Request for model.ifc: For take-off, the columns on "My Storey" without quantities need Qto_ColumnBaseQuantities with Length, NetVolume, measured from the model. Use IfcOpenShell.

First a look at what the model holds.

```python
import ifcopenshell
import ifcopenshell.util.element
import ifcopenshell.util.unit

model = ifcopenshell.open("model.ifc")
print(model.schema)
for unit_type in ("LENGTHUNIT", "AREAUNIT", "VOLUMEUNIT"):
    print(unit_type, ifcopenshell.util.unit.calculate_unit_scale(model, unit_type))
storey = next(s for s in model.by_type("IfcBuildingStorey") if s.Name == "My Storey")
columns = [e for e in ifcopenshell.util.element.get_decomposition(storey) if e.is_a("IfcColumn")]
for e in sorted(columns, key=lambda e: e.id()):
    print(e.id(), e.is_a(), e.Name, list(ifcopenshell.util.element.get_psets(e, qtos_only=True)), sep=" | ")
```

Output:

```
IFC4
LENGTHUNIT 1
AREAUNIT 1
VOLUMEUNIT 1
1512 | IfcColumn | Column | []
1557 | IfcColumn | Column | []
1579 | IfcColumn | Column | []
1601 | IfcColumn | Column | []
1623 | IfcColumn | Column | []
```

```python
import ifcopenshell
import ifcopenshell.api.pset
import ifcopenshell.geom
import ifcopenshell.util.element
import ifcopenshell.util.shape
import ifcopenshell.util.unit

model = ifcopenshell.open("model.ifc")
unit_scale = ifcopenshell.util.unit.calculate_unit_scale(model)
volume_scale = ifcopenshell.util.unit.calculate_unit_scale(model, "VOLUMEUNIT")
settings = ifcopenshell.geom.settings()

storey = next(s for s in model.by_type("IfcBuildingStorey") if s.Name == "My Storey")
columns = [e for e in ifcopenshell.util.element.get_decomposition(storey) if e.is_a("IfcColumn")]

for e in sorted(columns, key=lambda e: e.id()):
    if ifcopenshell.util.element.get_psets(e, qtos_only=True, should_inherit=False):
        continue
    # Geometry comes back in metres, in the element's own axes.
    shape = ifcopenshell.geom.create_shape(settings, e)
    values = {
        "Length": ifcopenshell.util.shape.get_z(shape.geometry) / unit_scale,
        "NetVolume": ifcopenshell.util.shape.get_volume(shape.geometry) / volume_scale,
    }
    qto = ifcopenshell.api.pset.add_qto(model, product=e, name="Qto_ColumnBaseQuantities")
    ifcopenshell.api.pset.edit_qto(model, qto=qto, properties=values)
    print(e.id(), {k: round(v, 3) for k, v in values.items()})

model.write("model-out.ifc")
```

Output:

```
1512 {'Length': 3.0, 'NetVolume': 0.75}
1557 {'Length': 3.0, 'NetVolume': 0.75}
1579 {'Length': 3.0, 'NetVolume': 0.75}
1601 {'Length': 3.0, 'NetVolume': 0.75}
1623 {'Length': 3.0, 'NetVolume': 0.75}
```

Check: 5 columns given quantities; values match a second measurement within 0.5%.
